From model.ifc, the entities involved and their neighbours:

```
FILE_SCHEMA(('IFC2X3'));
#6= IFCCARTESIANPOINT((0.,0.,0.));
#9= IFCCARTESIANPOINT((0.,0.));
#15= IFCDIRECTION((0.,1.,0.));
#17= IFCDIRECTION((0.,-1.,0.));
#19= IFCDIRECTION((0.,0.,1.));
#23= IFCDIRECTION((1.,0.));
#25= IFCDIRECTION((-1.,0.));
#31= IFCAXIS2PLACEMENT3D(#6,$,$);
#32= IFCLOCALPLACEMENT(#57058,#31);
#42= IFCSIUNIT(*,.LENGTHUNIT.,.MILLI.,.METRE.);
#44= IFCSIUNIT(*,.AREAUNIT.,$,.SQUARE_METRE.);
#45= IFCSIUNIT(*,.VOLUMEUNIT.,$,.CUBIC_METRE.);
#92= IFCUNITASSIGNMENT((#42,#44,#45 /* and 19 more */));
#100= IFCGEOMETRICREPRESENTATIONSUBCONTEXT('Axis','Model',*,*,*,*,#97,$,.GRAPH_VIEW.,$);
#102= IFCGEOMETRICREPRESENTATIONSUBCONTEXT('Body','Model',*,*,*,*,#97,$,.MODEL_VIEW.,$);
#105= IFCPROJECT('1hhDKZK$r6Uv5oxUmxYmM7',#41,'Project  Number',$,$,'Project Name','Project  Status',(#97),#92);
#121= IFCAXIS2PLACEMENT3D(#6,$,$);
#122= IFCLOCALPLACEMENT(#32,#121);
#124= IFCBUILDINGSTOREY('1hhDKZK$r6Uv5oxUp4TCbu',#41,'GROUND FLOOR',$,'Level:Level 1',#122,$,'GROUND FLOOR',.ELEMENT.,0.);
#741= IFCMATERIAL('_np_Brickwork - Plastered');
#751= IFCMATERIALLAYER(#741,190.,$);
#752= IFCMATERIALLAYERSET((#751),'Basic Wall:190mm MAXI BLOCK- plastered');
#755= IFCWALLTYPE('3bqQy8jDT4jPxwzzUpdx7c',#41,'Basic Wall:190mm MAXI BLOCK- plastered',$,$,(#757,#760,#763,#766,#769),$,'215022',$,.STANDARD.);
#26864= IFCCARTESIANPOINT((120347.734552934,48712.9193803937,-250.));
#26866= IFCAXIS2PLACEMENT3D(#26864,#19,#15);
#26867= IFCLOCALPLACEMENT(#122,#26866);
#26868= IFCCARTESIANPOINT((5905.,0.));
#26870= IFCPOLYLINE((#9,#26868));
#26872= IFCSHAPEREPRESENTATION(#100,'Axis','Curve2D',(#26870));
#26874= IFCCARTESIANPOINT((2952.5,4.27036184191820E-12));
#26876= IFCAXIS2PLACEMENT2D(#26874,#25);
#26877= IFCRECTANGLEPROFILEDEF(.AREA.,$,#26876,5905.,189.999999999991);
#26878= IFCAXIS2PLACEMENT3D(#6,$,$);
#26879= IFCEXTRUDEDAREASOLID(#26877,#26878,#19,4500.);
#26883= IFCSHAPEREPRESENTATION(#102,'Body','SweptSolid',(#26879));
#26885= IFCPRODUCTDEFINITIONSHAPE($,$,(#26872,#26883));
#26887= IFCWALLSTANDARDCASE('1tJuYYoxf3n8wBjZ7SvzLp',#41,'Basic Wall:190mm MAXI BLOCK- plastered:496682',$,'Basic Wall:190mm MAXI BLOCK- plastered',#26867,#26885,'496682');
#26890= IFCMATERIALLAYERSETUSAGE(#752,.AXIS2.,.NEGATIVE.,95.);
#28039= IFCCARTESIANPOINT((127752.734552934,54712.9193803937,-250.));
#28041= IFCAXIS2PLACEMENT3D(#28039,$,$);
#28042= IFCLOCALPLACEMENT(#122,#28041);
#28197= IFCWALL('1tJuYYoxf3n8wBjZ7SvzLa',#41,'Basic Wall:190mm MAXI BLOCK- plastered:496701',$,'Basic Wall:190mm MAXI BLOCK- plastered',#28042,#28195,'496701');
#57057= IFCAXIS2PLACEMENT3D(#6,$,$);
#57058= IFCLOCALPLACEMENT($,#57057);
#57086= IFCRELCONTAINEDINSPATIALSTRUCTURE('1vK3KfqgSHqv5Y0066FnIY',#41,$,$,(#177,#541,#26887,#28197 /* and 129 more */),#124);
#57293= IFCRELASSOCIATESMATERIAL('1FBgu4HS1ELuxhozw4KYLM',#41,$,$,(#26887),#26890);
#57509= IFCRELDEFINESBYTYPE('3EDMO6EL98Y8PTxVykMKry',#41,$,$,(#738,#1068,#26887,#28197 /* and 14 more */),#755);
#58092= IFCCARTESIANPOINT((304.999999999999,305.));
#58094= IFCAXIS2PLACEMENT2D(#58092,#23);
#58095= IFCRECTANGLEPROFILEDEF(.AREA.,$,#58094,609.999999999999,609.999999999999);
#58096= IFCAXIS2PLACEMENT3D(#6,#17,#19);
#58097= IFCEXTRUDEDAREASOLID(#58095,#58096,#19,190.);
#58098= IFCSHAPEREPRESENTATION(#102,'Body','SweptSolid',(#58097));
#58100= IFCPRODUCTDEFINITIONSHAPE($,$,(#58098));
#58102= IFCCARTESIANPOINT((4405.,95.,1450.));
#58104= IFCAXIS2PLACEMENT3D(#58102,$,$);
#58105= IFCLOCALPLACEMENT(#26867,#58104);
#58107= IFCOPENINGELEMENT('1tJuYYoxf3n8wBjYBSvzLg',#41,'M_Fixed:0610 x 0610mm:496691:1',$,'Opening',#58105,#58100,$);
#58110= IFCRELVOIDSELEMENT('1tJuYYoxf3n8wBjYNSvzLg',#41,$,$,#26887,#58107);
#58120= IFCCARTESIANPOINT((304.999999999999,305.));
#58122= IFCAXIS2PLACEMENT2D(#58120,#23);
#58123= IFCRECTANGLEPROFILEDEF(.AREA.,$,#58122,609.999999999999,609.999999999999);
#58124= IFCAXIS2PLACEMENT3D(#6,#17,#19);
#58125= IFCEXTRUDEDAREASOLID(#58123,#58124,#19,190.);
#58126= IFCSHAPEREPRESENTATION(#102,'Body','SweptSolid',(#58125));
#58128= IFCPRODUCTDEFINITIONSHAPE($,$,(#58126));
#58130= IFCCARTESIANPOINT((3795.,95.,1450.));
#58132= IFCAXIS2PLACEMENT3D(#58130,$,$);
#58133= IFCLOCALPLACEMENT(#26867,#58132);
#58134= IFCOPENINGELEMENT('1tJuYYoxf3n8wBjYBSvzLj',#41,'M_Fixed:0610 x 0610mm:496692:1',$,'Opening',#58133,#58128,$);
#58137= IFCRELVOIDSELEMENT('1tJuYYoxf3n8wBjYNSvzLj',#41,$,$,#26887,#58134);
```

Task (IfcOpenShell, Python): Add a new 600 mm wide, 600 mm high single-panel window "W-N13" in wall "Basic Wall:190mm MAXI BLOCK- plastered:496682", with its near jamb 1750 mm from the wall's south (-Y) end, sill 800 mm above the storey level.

```python
import numpy as np
import ifcopenshell
import ifcopenshell.api.feature
import ifcopenshell.api.geometry
import ifcopenshell.api.root
import ifcopenshell.api.spatial
import ifcopenshell.api.type
import ifcopenshell.geom
import ifcopenshell.util.element
import ifcopenshell.util.placement
import ifcopenshell.util.representation
import ifcopenshell.util.shape
import ifcopenshell.util.unit

model = ifcopenshell.open("model.ifc")
unit_scale = ifcopenshell.util.unit.calculate_unit_scale(model)
settings = ifcopenshell.geom.settings()


def volume(element):
    """Net volume in cubic metres, openings subtracted."""
    shape = ifcopenshell.geom.create_shape(settings, element)
    return ifcopenshell.util.shape.get_volume(shape.geometry)


wall = model.by_guid("1tJuYYoxf3n8wBjZ7SvzLp")
storey = ifcopenshell.util.element.get_container(wall, ifc_class="IfcBuildingStorey")
context = ifcopenshell.util.representation.get_context(model, "Model", "Body", "MODEL_VIEW")
before = volume(wall)

width, height, from_end, sill = 0.6, 0.6, 1.75, 0.8  # metres

# The wall runs along its own X axis, and the end named is its -X end.
wall_shape = ifcopenshell.geom.create_shape(settings, wall)
x, y, z = ifcopenshell.util.shape.get_vertices(wall_shape.geometry).T
start = x.min() + from_end
face, thickness = float(y.min()), float(y.max() - y.min())
wall_matrix = ifcopenshell.util.placement.get_local_placement(wall.ObjectPlacement)
level = ifcopenshell.util.placement.get_local_placement(storey.ObjectPlacement)[2, 3]


def in_wall(x, y):
    """Placement at x, y metres in the wall's axes, at sill height."""
    matrix = wall_matrix.copy()
    matrix[:, 3] = wall_matrix @ np.array([x / unit_scale, y / unit_scale, 0.0, 1.0])
    matrix[2, 3] = level + sill / unit_scale
    return matrix


# Opening: a box that overshoots both wall faces by 50 mm.
opening = ifcopenshell.api.root.create_entity(model, ifc_class="IfcOpeningElement")
box = ifcopenshell.api.geometry.add_wall_representation(
    model, context=context, length=width, height=height, thickness=thickness + 0.1
)
ifcopenshell.api.geometry.assign_representation(model, product=opening, representation=box)
ifcopenshell.api.geometry.edit_object_placement(model, product=opening, matrix=in_wall(start, face - 0.05), is_si=False)
ifcopenshell.api.feature.add_feature(model, feature=opening, element=wall)

window = ifcopenshell.api.root.create_entity(model, ifc_class="IfcWindow", name="W-N13")
window.OverallWidth, window.OverallHeight = width / unit_scale, height / unit_scale
body = ifcopenshell.api.geometry.add_window_representation(
    model,
    context=context,
    overall_width=window.OverallWidth,
    overall_height=window.OverallHeight,
    partition_type="SINGLE_PANEL",
)
ifcopenshell.api.geometry.assign_representation(model, product=window, representation=body)
ifcopenshell.api.spatial.assign_container(model, products=[window], relating_structure=storey)
fills = ifcopenshell.api.feature.add_filling(model, opening=opening, element=window)
fills.OwnerHistory = window.OwnerHistory  # required in IFC2X3

# IFC2X3 keeps the operation on the window style.
style = ifcopenshell.api.root.create_entity(model, ifc_class="IfcWindowStyle", name="W-N13")
style.OperationType, style.ConstructionType = "SINGLE_PANEL", "NOTDEFINED"
style.ParameterTakesPrecedence = style.Sizeable = False
ifcopenshell.api.type.assign_type(model, related_objects=[window], relating_type=style)

# Centre the window in the wall's thickness.
ifcopenshell.api.geometry.edit_object_placement(model, product=window, matrix=in_wall(start, face), is_si=False)
window_shape = ifcopenshell.geom.create_shape(settings, window)
depth = ifcopenshell.util.shape.get_vertices(window_shape.geometry)[:, 1]
offset = face + thickness / 2 - (depth.min() + depth.max()) / 2
ifcopenshell.api.geometry.edit_object_placement(model, product=window, matrix=in_wall(start, offset), is_si=False)

after = volume(wall)

print(f"wall volume {before:.3f} -> {after:.3f} m3")

model.write("model_edited.ifc")
```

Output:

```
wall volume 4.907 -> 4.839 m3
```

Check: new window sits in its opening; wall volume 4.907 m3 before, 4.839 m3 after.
